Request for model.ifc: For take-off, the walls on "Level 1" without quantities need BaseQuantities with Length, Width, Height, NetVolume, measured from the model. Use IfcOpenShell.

First a look at what the model holds.

```python
import ifcopenshell
import ifcopenshell.util.element
import ifcopenshell.util.unit

model = ifcopenshell.open("model.ifc")
print(model.schema)
for unit_type in ("LENGTHUNIT", "AREAUNIT", "VOLUMEUNIT"):
    print(unit_type, ifcopenshell.util.unit.calculate_unit_scale(model, unit_type))
storey = next(s for s in model.by_type("IfcBuildingStorey") if s.Name == "Level 1")
walls = [e for e in ifcopenshell.util.element.get_decomposition(storey) if e.is_a("IfcWall")]
for e in sorted(walls, key=lambda e: e.id()):
    print(e.id(), e.is_a(), e.Name, list(ifcopenshell.util.element.get_psets(e, qtos_only=True)), sep=" | ")
```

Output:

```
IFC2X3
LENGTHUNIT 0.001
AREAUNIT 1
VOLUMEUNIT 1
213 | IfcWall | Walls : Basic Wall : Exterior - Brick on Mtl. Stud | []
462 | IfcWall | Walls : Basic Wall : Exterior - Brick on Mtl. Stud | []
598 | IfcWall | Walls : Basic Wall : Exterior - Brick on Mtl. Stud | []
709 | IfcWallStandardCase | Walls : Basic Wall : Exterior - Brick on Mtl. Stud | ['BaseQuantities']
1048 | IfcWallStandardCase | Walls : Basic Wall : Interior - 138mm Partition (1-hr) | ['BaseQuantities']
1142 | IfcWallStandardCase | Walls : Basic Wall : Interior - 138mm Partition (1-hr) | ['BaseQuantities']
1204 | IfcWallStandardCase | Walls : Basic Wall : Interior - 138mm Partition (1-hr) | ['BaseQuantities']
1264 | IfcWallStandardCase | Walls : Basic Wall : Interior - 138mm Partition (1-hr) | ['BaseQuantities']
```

```python
import ifcopenshell
import ifcopenshell.api.pset
import ifcopenshell.geom
import ifcopenshell.util.element
import ifcopenshell.util.shape
import ifcopenshell.util.unit

model = ifcopenshell.open("model.ifc")
unit_scale = ifcopenshell.util.unit.calculate_unit_scale(model)
volume_scale = ifcopenshell.util.unit.calculate_unit_scale(model, "VOLUMEUNIT")
settings = ifcopenshell.geom.settings()

storey = next(s for s in model.by_type("IfcBuildingStorey") if s.Name == "Level 1")
walls = [e for e in ifcopenshell.util.element.get_decomposition(storey) if e.is_a("IfcWall")]

for e in sorted(walls, key=lambda e: e.id()):
    if ifcopenshell.util.element.get_psets(e, qtos_only=True, should_inherit=False):
        continue
    # Geometry comes back in metres, in the element's own axes.
    shape = ifcopenshell.geom.create_shape(settings, e)
    values = {
        "Length": ifcopenshell.util.shape.get_x(shape.geometry) / unit_scale,
        "Width": ifcopenshell.util.shape.get_y(shape.geometry) / unit_scale,
        "Height": ifcopenshell.util.shape.get_z(shape.geometry) / unit_scale,
        "NetVolume": ifcopenshell.util.shape.get_volume(shape.geometry) / volume_scale,
    }
    qto = ifcopenshell.api.pset.add_qto(model, product=e, name="BaseQuantities")
    ifcopenshell.api.pset.edit_qto(model, qto=qto, properties=values)
    print(e.id(), {k: round(v, 3) for k, v in values.items()})

model.write("model_v2.ifc")
```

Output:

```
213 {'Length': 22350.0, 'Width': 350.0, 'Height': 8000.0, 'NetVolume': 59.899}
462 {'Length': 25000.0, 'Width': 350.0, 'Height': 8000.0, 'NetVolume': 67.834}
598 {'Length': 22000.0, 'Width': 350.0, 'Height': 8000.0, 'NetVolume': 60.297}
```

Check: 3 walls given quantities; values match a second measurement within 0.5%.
